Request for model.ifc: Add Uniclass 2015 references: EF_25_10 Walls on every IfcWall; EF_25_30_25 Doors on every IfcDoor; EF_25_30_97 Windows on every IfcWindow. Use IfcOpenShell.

First a look at what the model holds.

```python
import ifcopenshell

model = ifcopenshell.open("model.ifc")
print(model.schema)
print("classifications:", [c.Name for c in model.by_type("IfcClassification")])
for ifc_class in ("IfcDoor", "IfcRoof", "IfcStair", "IfcWall", "IfcWindow"):
    print(ifc_class, len(model.by_type(ifc_class)))
```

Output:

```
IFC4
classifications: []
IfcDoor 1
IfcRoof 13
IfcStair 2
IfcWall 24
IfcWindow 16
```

```python
import ifcopenshell
import ifcopenshell.api.classification

model = ifcopenshell.open("model.ifc")

system = ifcopenshell.api.classification.add_classification(model, classification="Uniclass 2015")

codes = {
    "IfcWall": ("EF_25_10", "Walls"),
    "IfcDoor": ("EF_25_30_25", "Doors"),
    "IfcWindow": ("EF_25_30_97", "Windows"),
}
for ifc_class, (code, name) in codes.items():
    products = model.by_type(ifc_class)
    ifcopenshell.api.classification.add_reference(
        model, products=products, classification=system, identification=code, name=name
    )
    print(code, len(products))

model.write("model_edited.ifc")
```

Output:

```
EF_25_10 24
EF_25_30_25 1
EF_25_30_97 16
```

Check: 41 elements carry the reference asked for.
